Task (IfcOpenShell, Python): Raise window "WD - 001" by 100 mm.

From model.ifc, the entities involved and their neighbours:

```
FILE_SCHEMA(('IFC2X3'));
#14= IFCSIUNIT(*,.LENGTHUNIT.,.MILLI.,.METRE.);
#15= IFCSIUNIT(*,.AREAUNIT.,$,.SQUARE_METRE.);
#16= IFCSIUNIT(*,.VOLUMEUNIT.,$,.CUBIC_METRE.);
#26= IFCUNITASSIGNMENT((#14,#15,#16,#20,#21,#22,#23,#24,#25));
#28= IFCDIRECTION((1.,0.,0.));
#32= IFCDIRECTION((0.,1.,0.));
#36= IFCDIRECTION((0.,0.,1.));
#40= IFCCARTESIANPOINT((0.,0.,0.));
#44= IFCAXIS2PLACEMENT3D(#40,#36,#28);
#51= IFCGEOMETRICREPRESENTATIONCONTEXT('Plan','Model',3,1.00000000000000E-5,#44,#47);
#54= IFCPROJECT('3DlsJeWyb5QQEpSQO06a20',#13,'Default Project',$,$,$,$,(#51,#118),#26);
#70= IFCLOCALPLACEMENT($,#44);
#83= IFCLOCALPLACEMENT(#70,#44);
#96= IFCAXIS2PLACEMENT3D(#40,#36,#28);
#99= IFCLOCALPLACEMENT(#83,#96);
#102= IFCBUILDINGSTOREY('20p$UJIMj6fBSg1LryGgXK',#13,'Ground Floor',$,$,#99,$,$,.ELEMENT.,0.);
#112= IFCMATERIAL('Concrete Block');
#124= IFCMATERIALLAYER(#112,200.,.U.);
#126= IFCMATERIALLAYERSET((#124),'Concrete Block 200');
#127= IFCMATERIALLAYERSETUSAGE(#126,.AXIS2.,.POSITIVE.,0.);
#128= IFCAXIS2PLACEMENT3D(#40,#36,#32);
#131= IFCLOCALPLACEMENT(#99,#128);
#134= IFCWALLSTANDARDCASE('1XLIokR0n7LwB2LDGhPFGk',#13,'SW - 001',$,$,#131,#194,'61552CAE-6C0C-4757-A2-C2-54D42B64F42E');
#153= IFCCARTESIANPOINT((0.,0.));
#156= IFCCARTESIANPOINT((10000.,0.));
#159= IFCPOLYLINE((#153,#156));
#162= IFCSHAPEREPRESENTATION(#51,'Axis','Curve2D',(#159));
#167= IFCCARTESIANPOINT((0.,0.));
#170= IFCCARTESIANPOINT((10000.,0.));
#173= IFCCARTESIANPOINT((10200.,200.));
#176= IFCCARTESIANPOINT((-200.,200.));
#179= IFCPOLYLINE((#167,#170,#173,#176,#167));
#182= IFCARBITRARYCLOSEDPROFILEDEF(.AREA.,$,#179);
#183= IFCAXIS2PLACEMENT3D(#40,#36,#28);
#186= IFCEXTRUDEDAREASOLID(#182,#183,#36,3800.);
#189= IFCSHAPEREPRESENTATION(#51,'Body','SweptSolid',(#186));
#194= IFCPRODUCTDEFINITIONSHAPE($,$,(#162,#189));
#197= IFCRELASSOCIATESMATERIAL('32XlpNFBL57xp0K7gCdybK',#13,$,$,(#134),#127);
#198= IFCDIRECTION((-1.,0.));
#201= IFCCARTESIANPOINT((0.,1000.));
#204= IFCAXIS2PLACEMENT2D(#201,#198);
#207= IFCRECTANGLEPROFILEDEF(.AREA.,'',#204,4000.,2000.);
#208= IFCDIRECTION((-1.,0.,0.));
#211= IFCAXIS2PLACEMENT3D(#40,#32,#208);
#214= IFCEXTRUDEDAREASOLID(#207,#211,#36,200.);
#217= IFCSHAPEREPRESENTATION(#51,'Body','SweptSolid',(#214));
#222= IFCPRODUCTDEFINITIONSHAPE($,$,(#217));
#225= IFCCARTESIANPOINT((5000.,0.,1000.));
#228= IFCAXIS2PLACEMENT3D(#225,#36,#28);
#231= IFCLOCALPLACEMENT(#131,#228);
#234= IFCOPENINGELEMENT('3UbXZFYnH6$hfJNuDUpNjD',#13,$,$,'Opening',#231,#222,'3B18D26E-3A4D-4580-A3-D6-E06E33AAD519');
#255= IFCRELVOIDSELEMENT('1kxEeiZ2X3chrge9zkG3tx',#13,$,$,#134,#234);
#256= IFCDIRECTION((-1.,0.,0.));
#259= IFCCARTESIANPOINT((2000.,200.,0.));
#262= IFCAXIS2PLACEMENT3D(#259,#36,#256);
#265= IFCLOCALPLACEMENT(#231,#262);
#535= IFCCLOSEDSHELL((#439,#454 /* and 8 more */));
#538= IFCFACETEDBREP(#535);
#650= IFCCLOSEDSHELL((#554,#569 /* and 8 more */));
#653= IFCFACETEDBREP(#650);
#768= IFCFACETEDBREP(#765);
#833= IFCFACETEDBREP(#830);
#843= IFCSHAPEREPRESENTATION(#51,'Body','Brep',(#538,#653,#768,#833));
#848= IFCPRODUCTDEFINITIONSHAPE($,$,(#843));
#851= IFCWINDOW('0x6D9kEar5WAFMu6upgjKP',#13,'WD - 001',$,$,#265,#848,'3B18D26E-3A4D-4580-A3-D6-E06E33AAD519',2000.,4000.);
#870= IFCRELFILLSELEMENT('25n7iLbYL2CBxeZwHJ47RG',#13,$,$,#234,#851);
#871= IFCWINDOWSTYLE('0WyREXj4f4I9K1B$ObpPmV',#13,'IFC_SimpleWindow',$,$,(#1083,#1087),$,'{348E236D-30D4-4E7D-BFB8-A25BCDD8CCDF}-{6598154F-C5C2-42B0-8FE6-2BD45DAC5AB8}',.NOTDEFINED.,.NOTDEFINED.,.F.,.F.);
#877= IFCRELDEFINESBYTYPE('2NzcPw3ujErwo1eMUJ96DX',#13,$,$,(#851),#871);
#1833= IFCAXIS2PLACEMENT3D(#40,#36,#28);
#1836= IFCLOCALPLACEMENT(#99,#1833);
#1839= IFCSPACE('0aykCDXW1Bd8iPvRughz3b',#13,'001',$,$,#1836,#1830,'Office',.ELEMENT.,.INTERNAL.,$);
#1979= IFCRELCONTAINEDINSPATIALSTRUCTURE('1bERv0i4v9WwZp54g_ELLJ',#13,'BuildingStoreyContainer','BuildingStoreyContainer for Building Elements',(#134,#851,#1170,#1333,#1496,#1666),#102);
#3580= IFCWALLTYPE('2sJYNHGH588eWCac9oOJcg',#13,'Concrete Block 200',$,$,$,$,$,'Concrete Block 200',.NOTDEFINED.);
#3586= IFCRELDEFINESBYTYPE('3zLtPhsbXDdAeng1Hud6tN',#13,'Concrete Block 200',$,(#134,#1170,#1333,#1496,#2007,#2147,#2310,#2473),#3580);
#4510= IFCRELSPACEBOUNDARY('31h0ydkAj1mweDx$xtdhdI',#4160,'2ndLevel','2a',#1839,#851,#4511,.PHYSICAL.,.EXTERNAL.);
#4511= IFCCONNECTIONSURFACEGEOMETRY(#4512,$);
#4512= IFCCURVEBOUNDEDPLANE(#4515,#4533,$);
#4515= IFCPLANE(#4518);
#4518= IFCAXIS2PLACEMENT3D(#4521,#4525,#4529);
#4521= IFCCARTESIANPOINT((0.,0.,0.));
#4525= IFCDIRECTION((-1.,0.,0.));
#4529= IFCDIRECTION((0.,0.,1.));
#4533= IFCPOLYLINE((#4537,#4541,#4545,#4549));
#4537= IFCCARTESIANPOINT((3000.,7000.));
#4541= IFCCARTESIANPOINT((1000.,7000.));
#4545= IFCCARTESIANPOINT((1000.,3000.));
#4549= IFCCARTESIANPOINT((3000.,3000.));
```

```python
import numpy as np
import ifcopenshell
import ifcopenshell.api.geometry
import ifcopenshell.util.placement
import ifcopenshell.util.unit

model = ifcopenshell.open("model.ifc")
unit_scale = ifcopenshell.util.unit.calculate_unit_scale(model)

window = model.by_id(851)
opening = window.FillsVoids[0].RelatingOpeningElement
dz = 100.0

shift = np.array([0.0, 0.0, dz])
# The window is placed relative to its opening, so it follows when the opening moves.
matrix = ifcopenshell.util.placement.get_local_placement(opening.ObjectPlacement)
matrix[:3, 3] += shift
ifcopenshell.api.geometry.edit_object_placement(
    model, product=opening, matrix=matrix, is_si=False, should_transform_children=True
)

# Space boundary surfaces are stored in each space's coordinates; move them too.
for rel in window.ProvidesBoundaries:
    if not rel.ConnectionGeometry:
        continue
    surface = rel.ConnectionGeometry.SurfaceOnRelatingElement.BasisSurface
    space_matrix = ifcopenshell.util.placement.get_local_placement(rel.RelatingSpace.ObjectPlacement)
    point = np.array(surface.Position.Location.Coordinates) + space_matrix[:3, :3].T @ shift
    surface.Position = model.createIfcAxis2Placement3D(
        model.createIfcCartesianPoint(point.tolist()), surface.Position.Axis, surface.Position.RefDirection
    )

print(f"moved by {dz * unit_scale:+.3f} m")

model.write("model_updated.ifc")
```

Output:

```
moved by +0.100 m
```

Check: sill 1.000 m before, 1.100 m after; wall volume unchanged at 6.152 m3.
